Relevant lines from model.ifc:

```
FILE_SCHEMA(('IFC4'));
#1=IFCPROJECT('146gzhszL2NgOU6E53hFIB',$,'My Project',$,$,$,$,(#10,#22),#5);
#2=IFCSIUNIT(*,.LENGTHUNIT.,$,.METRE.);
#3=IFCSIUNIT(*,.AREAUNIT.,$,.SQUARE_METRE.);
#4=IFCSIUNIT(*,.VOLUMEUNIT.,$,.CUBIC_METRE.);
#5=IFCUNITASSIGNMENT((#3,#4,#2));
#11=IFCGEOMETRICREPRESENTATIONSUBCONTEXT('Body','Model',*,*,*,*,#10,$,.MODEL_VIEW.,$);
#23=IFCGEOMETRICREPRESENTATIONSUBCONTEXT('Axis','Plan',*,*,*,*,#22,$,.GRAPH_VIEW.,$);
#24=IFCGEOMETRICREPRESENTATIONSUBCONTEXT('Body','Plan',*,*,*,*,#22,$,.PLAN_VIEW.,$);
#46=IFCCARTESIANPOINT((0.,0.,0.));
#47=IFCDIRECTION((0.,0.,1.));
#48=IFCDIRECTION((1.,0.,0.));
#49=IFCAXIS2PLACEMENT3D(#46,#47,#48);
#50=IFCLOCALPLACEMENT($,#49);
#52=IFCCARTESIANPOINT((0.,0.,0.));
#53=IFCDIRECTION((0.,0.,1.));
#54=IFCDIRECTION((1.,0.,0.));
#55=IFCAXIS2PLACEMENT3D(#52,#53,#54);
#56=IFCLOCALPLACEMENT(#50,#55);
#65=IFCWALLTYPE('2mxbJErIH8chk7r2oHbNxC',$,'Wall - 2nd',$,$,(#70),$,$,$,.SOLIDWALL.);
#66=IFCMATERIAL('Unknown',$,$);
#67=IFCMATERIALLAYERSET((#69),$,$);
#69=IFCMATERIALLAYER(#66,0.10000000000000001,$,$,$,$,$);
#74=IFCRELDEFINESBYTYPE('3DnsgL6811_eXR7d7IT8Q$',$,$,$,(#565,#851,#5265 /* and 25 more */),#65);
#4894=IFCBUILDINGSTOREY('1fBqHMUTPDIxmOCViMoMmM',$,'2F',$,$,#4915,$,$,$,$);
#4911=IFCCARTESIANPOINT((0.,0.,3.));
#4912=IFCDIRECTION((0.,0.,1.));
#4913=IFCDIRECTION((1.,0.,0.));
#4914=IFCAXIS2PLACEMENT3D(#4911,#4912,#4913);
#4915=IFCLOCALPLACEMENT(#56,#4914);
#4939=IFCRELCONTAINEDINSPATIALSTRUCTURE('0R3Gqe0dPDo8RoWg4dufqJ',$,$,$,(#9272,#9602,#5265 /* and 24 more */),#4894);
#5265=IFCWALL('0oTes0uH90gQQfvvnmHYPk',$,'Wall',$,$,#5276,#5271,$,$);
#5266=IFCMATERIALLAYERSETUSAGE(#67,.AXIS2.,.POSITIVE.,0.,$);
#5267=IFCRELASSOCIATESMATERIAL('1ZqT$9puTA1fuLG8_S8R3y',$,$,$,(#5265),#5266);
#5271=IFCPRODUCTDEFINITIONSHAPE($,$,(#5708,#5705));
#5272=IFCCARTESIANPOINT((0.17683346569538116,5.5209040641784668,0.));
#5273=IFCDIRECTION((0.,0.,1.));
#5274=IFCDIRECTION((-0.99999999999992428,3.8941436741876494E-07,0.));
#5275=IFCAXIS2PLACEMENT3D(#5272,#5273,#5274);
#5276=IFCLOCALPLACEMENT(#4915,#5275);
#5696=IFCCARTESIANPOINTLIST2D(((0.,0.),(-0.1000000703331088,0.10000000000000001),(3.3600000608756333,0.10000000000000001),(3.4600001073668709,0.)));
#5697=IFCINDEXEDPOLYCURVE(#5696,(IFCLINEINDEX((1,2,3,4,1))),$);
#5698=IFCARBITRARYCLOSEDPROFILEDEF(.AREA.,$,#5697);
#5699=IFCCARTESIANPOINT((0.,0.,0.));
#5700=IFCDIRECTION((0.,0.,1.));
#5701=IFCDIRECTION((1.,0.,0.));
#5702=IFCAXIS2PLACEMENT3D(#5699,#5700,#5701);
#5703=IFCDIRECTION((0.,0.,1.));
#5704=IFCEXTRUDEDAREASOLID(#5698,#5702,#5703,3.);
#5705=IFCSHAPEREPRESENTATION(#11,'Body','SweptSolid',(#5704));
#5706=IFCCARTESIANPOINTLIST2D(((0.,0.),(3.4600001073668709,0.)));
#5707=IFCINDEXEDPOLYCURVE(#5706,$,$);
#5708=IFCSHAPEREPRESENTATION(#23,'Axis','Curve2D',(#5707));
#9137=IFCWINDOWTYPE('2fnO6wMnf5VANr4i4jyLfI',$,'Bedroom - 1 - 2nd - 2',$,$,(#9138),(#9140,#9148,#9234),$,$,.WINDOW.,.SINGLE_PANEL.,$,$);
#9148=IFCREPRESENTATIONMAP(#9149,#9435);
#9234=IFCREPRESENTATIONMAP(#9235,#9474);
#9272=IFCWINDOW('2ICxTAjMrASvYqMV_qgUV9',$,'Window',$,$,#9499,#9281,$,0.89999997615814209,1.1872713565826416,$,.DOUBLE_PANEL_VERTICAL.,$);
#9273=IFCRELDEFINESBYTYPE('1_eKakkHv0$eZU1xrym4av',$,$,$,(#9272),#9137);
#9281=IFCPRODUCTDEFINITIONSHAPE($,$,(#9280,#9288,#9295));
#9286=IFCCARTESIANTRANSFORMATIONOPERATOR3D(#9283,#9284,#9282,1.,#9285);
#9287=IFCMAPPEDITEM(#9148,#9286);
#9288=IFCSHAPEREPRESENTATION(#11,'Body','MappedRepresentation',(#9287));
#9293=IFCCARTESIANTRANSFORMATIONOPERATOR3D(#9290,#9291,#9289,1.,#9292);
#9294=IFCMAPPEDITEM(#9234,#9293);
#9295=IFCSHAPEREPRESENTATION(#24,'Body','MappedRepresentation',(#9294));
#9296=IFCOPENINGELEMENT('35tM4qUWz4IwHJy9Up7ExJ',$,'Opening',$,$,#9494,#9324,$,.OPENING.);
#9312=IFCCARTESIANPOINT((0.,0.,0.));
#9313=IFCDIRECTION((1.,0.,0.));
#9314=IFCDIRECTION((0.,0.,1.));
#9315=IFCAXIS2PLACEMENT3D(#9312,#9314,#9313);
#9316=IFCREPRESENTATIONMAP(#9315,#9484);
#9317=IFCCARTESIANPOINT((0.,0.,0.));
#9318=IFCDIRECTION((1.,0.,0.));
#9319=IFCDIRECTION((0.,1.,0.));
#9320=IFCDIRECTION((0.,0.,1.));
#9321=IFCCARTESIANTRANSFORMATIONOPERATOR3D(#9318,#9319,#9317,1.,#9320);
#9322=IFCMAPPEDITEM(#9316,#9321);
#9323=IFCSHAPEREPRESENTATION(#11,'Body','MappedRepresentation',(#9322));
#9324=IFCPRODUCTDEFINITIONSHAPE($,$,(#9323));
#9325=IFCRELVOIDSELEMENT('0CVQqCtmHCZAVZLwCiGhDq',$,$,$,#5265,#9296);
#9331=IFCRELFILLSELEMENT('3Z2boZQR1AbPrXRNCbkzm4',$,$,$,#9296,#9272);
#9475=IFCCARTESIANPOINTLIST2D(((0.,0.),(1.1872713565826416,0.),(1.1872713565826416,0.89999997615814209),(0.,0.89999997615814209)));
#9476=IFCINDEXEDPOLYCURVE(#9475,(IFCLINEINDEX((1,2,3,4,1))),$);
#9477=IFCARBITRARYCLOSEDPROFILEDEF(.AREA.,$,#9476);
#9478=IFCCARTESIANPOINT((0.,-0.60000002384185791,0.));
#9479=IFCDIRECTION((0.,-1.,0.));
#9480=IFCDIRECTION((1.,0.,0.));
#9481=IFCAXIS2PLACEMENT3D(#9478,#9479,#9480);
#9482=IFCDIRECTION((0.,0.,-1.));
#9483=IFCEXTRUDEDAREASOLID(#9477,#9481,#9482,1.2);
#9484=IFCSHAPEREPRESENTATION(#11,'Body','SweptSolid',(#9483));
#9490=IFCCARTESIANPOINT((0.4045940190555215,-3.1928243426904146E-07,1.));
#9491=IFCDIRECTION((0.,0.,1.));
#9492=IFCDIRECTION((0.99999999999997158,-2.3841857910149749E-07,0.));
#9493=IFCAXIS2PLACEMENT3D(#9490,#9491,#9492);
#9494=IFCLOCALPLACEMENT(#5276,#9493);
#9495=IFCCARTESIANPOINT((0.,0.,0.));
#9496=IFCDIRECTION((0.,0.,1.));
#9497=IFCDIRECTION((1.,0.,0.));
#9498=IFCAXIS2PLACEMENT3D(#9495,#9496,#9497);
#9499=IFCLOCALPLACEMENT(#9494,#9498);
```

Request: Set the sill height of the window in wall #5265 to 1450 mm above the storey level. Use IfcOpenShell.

```python
import numpy as np
import ifcopenshell
import ifcopenshell.api.geometry
import ifcopenshell.geom
import ifcopenshell.util.element
import ifcopenshell.util.placement
import ifcopenshell.util.shape
import ifcopenshell.util.unit

model = ifcopenshell.open("model.ifc")
unit_scale = ifcopenshell.util.unit.calculate_unit_scale(model)

window = model.by_guid("2ICxTAjMrASvYqMV_qgUV9")
opening = window.FillsVoids[0].RelatingOpeningElement
storey = ifcopenshell.util.element.get_container(window, ifc_class="IfcBuildingStorey")
level = ifcopenshell.util.placement.get_local_placement(storey.ObjectPlacement)[2, 3]

# The opening's origin need not be at the sill, so measure its lowest point.
shape = ifcopenshell.geom.create_shape(ifcopenshell.geom.settings(), opening)
bottom = ifcopenshell.util.shape.get_shape_bottom_elevation(shape, shape.geometry) / unit_scale
dz = level + 1.45 - bottom

shift = np.array([0.0, 0.0, dz])
# The window is placed relative to its opening, so it follows when the opening moves.
matrix = ifcopenshell.util.placement.get_local_placement(opening.ObjectPlacement)
matrix[:3, 3] += shift
ifcopenshell.api.geometry.edit_object_placement(
    model, product=opening, matrix=matrix, is_si=False, should_transform_children=True
)

print(f"moved by {dz * unit_scale:+.3f} m")

model.write("model_rev.ifc")
```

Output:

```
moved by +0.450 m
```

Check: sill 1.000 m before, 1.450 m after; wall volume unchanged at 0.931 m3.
